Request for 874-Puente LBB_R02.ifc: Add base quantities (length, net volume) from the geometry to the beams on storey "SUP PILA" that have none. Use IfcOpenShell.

First a look at what the model holds.

```python
import ifcopenshell
import ifcopenshell.util.element
import ifcopenshell.util.unit

model = ifcopenshell.open("874-Puente LBB_R02.ifc")
print(model.schema)
for unit_type in ("LENGTHUNIT", "AREAUNIT", "VOLUMEUNIT"):
    print(unit_type, ifcopenshell.util.unit.calculate_unit_scale(model, unit_type))
storey = next(s for s in model.by_type("IfcBuildingStorey") if s.Name == "SUP PILA")
beams = [e for e in ifcopenshell.util.element.get_decomposition(storey) if e.is_a("IfcBeam")]
for e in sorted(beams, key=lambda e: e.id()):
    print(e.id(), e.is_a(), e.Name, list(ifcopenshell.util.element.get_psets(e, qtos_only=True)), sep=" | ")
```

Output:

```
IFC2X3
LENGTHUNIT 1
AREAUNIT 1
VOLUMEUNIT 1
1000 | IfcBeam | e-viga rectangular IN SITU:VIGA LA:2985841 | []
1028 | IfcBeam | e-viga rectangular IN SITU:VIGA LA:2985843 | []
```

```python
import ifcopenshell
import ifcopenshell.api.pset
import ifcopenshell.geom
import ifcopenshell.util.element
import ifcopenshell.util.shape
import ifcopenshell.util.unit

model = ifcopenshell.open("874-Puente LBB_R02.ifc")
unit_scale = ifcopenshell.util.unit.calculate_unit_scale(model)
volume_scale = ifcopenshell.util.unit.calculate_unit_scale(model, "VOLUMEUNIT")
settings = ifcopenshell.geom.settings()

storey = next(s for s in model.by_type("IfcBuildingStorey") if s.Name == "SUP PILA")
beams = [e for e in ifcopenshell.util.element.get_decomposition(storey) if e.is_a("IfcBeam")]

for e in sorted(beams, key=lambda e: e.id()):
    if ifcopenshell.util.element.get_psets(e, qtos_only=True, should_inherit=False):
        continue
    # Geometry comes back in metres, in the element's own axes.
    shape = ifcopenshell.geom.create_shape(settings, e)
    values = {
        "Length": ifcopenshell.util.shape.get_max_xyz(shape.geometry) / unit_scale,
        "NetVolume": ifcopenshell.util.shape.get_volume(shape.geometry) / volume_scale,
    }
    qto = ifcopenshell.api.pset.add_qto(model, product=e, name="BaseQuantities")
    ifcopenshell.api.pset.edit_qto(model, qto=qto, properties=values)
    print(e.id(), {k: round(v, 3) for k, v in values.items()})

model.write("874-Puente LBB_R02_rev.ifc")
```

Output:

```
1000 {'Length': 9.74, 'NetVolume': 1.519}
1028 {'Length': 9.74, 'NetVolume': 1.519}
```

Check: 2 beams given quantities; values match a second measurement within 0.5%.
